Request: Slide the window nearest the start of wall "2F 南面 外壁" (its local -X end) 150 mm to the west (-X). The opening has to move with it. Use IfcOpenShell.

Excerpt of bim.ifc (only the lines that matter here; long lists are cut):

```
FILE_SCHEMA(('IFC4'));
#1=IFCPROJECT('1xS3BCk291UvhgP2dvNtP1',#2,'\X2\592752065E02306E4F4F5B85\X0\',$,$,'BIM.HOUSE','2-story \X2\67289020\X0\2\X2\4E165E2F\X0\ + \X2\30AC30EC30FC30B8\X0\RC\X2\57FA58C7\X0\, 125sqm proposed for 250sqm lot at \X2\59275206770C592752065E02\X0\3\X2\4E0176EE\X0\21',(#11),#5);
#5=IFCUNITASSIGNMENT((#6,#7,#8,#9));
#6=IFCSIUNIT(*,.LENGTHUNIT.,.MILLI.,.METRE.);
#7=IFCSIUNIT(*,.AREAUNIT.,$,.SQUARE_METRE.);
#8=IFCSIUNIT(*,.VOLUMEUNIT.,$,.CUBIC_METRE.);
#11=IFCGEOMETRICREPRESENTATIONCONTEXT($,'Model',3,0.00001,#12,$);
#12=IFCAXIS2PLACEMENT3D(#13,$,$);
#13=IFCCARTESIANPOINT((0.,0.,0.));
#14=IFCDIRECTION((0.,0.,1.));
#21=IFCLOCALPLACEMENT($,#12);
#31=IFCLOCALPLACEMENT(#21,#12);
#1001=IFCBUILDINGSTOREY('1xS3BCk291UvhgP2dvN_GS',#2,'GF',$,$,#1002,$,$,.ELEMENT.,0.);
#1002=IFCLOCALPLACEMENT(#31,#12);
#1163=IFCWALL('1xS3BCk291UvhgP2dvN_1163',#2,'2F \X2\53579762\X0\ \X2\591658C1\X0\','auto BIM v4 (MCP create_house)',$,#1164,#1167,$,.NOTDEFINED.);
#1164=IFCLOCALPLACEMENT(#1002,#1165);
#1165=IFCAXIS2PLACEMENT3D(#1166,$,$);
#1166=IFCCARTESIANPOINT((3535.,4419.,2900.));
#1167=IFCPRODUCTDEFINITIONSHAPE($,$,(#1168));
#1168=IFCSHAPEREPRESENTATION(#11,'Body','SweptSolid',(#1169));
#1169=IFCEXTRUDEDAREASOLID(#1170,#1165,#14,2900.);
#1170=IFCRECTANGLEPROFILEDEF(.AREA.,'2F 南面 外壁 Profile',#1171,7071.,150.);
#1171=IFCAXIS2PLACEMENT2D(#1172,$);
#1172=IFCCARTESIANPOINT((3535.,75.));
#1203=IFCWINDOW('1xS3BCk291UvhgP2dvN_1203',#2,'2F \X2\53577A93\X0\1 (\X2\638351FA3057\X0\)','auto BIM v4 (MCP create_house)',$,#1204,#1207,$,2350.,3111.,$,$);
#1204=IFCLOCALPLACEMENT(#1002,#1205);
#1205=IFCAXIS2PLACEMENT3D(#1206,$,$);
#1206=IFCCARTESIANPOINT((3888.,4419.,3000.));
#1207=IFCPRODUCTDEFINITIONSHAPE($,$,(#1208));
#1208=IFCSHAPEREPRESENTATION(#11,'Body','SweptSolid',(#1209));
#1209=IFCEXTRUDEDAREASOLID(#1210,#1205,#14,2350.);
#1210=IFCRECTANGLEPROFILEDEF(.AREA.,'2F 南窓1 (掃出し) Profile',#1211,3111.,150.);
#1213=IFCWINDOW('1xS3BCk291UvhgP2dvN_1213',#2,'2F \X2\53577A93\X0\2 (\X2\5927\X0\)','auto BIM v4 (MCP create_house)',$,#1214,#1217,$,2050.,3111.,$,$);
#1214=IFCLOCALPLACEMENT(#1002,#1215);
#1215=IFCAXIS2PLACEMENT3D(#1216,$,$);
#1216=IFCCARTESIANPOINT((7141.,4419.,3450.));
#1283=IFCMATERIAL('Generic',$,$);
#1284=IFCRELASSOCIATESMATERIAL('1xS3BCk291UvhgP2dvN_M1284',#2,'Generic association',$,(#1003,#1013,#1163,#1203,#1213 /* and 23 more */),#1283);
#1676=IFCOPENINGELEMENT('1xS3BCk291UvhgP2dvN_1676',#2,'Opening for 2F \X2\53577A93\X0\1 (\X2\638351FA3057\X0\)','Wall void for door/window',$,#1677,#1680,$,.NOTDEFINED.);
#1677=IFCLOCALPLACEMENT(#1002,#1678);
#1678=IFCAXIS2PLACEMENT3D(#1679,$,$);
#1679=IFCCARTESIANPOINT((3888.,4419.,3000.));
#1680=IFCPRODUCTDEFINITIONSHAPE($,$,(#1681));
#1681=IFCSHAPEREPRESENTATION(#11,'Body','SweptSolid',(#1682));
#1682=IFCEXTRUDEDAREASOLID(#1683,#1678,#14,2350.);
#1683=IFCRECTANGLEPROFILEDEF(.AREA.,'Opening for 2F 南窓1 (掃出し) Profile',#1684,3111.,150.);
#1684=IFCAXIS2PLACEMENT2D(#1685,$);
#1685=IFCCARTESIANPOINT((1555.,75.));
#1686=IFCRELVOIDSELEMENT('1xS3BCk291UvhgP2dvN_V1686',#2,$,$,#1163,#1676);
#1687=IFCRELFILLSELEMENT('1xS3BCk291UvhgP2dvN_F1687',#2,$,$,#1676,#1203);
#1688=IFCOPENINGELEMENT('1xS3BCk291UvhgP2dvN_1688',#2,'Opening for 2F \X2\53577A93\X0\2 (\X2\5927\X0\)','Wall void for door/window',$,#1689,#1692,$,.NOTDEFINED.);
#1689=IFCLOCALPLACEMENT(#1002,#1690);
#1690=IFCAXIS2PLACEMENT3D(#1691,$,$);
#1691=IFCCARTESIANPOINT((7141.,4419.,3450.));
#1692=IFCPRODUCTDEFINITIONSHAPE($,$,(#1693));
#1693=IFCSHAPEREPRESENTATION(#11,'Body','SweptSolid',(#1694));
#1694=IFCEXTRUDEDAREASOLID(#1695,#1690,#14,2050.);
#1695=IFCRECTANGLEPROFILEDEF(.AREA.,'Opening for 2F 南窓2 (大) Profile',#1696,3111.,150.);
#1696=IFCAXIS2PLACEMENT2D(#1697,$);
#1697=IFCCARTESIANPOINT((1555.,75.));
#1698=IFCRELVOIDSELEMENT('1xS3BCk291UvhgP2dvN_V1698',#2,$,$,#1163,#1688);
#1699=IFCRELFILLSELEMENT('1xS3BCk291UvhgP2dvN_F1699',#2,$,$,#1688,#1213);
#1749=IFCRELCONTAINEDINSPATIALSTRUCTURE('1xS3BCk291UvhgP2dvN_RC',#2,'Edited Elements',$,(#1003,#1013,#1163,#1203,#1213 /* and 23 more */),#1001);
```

```python
import ifcopenshell
import ifcopenshell.api.geometry
import ifcopenshell.util.placement
import ifcopenshell.util.unit

model = ifcopenshell.open("bim.ifc")
unit_scale = ifcopenshell.util.unit.calculate_unit_scale(model)

window = model.by_guid("1xS3BCk291UvhgP2dvN_1203")
opening = window.FillsVoids[0].RelatingOpeningElement
wall = opening.VoidsElements[0].RelatingBuildingElement

wall_matrix = ifcopenshell.util.placement.get_local_placement(wall.ObjectPlacement)
shift = wall_matrix[:3, 0] * -0.15 / unit_scale
before = ifcopenshell.util.placement.get_local_placement(window.ObjectPlacement)[:3, 3].copy()

# The window is not placed relative to its opening, so move both.
for product in (opening, window):
    matrix = ifcopenshell.util.placement.get_local_placement(product.ObjectPlacement)
    matrix[:3, 3] += shift
    ifcopenshell.api.geometry.edit_object_placement(model, product=product, matrix=matrix, is_si=False)

after = ifcopenshell.util.placement.get_local_placement(window.ObjectPlacement)[:3, 3]
print("window moved by", (after - before).round(3) + 0.0)

model.write("bim_rev.ifc")
```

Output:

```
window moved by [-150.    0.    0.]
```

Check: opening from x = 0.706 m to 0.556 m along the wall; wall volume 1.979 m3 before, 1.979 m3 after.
